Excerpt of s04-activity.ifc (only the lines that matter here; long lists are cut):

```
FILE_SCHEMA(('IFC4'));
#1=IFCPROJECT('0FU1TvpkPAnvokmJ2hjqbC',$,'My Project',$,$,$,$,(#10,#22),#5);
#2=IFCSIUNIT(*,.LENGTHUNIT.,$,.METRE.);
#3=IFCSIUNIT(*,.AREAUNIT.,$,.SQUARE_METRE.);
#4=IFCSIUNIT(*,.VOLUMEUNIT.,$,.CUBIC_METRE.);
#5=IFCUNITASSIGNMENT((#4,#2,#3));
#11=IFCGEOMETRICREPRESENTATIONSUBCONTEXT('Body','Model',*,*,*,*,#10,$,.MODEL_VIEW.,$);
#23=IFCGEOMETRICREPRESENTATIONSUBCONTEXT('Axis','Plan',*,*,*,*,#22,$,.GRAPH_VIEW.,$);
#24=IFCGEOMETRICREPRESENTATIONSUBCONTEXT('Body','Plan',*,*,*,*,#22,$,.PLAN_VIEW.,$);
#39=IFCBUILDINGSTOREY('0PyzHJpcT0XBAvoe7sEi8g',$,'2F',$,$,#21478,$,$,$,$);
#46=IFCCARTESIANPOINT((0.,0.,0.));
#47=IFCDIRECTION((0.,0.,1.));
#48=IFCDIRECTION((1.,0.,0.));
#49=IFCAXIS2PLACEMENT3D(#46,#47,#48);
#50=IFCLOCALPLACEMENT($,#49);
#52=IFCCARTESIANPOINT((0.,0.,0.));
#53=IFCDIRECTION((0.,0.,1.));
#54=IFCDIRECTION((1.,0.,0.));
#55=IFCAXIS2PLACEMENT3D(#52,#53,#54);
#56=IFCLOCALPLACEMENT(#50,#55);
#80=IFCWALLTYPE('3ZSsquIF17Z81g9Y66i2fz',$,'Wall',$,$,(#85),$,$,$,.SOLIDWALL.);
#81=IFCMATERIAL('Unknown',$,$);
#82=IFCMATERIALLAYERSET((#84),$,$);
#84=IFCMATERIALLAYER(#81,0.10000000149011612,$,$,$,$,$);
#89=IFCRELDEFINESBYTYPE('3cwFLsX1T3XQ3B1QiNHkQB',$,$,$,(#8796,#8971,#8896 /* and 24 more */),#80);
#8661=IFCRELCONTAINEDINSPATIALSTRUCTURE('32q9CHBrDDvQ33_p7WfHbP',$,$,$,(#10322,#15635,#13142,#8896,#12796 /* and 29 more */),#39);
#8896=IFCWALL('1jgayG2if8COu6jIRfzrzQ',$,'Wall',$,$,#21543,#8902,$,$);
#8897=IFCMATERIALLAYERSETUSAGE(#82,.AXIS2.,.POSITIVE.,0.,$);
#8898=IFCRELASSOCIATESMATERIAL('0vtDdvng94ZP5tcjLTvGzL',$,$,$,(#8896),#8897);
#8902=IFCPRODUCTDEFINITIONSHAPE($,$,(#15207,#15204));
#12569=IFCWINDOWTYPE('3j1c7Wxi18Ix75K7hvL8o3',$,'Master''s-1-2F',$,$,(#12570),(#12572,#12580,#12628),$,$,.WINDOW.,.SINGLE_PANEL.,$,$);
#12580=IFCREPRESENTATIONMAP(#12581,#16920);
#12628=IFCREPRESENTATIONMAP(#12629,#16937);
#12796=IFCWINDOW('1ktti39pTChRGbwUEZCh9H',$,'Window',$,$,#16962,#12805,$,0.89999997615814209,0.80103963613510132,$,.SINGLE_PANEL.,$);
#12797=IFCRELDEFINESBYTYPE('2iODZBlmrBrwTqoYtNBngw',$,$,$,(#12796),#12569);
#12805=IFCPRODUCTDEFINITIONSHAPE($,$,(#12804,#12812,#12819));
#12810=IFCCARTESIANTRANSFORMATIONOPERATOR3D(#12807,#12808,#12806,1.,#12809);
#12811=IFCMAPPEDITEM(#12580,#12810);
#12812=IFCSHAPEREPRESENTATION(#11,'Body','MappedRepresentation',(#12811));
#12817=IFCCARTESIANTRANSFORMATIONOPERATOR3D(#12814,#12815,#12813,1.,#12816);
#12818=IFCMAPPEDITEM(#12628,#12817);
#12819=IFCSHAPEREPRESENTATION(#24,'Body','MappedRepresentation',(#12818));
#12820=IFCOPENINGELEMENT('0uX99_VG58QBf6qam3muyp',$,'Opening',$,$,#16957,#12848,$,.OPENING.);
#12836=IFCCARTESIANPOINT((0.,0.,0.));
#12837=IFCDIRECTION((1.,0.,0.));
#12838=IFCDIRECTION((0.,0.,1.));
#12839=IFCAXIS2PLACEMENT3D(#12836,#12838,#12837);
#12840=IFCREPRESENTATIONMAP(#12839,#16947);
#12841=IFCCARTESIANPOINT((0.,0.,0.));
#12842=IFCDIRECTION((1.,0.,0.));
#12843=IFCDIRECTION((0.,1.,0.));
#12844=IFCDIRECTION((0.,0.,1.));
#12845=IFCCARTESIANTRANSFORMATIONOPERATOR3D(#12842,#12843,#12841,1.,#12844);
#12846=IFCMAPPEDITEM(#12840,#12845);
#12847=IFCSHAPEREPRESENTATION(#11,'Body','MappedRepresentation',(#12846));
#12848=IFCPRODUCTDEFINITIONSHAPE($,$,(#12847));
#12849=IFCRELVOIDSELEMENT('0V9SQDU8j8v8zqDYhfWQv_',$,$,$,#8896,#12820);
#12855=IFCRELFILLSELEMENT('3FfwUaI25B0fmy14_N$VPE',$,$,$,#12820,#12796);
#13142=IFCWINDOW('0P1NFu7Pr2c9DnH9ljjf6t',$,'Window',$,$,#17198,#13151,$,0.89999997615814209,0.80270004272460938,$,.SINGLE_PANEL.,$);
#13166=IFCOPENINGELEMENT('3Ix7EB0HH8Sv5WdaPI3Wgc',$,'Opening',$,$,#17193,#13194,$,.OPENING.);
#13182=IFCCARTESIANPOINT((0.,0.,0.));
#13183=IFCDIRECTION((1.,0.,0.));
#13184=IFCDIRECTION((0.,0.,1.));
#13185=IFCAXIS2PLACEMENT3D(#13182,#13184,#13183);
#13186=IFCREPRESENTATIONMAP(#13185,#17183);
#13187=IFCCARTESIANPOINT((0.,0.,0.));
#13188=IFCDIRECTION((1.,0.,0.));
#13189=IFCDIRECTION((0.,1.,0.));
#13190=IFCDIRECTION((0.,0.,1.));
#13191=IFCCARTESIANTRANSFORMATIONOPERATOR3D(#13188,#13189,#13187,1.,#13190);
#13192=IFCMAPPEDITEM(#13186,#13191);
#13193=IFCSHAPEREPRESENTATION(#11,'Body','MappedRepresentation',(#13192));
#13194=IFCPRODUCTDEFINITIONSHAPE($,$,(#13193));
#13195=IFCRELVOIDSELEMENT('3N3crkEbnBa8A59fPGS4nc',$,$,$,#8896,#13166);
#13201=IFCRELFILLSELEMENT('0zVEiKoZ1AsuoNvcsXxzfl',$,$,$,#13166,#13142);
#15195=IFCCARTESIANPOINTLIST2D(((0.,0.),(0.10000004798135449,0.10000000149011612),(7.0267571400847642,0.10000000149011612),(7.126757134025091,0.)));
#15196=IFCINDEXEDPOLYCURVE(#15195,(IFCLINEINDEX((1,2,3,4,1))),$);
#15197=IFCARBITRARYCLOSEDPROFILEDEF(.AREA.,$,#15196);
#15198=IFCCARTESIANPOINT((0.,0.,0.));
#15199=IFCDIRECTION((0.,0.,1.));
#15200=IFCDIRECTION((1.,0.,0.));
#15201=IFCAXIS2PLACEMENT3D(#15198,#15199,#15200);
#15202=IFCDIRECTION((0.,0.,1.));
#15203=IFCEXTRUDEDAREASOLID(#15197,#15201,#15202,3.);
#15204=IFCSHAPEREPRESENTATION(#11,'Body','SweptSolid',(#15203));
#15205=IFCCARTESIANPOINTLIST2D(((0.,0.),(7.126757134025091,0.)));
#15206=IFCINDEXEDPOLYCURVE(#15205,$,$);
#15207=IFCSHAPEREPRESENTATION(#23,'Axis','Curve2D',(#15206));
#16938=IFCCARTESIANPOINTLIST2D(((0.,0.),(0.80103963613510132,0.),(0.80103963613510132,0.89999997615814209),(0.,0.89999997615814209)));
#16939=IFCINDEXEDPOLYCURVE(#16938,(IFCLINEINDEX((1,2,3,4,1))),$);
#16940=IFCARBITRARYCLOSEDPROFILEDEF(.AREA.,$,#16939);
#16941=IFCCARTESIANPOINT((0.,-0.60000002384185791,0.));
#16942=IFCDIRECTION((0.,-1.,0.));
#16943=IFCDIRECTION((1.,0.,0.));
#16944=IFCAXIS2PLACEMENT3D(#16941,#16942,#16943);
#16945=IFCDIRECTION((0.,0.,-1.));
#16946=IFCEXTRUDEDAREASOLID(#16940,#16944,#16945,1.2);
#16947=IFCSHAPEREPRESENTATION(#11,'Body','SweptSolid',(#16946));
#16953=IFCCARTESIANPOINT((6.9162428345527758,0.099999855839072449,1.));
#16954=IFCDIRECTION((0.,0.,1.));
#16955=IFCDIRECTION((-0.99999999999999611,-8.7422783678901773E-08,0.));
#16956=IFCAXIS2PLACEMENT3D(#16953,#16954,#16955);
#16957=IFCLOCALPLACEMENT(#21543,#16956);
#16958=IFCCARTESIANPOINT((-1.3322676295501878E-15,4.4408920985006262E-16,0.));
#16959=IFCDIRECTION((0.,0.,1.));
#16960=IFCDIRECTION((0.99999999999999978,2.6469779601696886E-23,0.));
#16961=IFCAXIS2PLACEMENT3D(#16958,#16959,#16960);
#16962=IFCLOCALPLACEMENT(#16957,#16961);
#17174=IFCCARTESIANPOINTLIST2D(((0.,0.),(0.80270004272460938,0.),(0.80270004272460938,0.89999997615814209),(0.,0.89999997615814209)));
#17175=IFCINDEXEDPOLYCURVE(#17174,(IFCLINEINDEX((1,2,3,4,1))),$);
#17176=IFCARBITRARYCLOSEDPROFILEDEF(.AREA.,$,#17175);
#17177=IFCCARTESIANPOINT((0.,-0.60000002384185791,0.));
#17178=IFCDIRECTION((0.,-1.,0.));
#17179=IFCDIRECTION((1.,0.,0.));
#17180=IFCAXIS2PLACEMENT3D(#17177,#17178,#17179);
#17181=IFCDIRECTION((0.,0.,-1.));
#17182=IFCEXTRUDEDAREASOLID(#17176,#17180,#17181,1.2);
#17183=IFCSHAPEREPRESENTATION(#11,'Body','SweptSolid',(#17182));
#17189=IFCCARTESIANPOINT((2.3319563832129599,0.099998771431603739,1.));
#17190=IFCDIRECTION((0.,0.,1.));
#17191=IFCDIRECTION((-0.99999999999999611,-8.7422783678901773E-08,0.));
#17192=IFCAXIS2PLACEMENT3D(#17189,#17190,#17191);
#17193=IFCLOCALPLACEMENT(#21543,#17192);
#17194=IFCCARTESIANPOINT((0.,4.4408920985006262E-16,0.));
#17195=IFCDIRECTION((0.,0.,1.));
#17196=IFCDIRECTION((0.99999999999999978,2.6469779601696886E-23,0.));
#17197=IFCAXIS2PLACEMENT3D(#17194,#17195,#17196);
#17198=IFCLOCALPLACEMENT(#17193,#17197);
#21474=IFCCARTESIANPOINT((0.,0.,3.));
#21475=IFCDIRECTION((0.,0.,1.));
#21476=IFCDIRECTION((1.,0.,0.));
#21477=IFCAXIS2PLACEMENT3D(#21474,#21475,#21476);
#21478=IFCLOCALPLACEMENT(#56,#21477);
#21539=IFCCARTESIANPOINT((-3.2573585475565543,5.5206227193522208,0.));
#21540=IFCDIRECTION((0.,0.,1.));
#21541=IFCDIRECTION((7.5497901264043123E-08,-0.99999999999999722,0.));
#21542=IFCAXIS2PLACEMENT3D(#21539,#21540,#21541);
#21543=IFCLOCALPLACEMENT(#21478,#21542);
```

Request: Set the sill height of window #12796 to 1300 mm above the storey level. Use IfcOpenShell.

```python
import numpy as np
import ifcopenshell
import ifcopenshell.api.geometry
import ifcopenshell.geom
import ifcopenshell.util.element
import ifcopenshell.util.placement
import ifcopenshell.util.shape
import ifcopenshell.util.unit

model = ifcopenshell.open("s04-activity.ifc")
unit_scale = ifcopenshell.util.unit.calculate_unit_scale(model)

window = model.by_guid("1ktti39pTChRGbwUEZCh9H")
opening = window.FillsVoids[0].RelatingOpeningElement
storey = ifcopenshell.util.element.get_container(window, ifc_class="IfcBuildingStorey")
level = ifcopenshell.util.placement.get_local_placement(storey.ObjectPlacement)[2, 3]

# The opening's origin need not be at the sill, so measure its lowest point.
shape = ifcopenshell.geom.create_shape(ifcopenshell.geom.settings(), opening)
bottom = ifcopenshell.util.shape.get_shape_bottom_elevation(shape, shape.geometry) / unit_scale
dz = level + 1.3 - bottom

shift = np.array([0.0, 0.0, dz])
# The window is placed relative to its opening, so it follows when the opening moves.
matrix = ifcopenshell.util.placement.get_local_placement(opening.ObjectPlacement)
matrix[:3, 3] += shift
ifcopenshell.api.geometry.edit_object_placement(
    model, product=opening, matrix=matrix, is_si=False, should_transform_children=True
)

print(f"moved by {dz * unit_scale:+.3f} m")

model.write("s04-activity-out.ifc")
```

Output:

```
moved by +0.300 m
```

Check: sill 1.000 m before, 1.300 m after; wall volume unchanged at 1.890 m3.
